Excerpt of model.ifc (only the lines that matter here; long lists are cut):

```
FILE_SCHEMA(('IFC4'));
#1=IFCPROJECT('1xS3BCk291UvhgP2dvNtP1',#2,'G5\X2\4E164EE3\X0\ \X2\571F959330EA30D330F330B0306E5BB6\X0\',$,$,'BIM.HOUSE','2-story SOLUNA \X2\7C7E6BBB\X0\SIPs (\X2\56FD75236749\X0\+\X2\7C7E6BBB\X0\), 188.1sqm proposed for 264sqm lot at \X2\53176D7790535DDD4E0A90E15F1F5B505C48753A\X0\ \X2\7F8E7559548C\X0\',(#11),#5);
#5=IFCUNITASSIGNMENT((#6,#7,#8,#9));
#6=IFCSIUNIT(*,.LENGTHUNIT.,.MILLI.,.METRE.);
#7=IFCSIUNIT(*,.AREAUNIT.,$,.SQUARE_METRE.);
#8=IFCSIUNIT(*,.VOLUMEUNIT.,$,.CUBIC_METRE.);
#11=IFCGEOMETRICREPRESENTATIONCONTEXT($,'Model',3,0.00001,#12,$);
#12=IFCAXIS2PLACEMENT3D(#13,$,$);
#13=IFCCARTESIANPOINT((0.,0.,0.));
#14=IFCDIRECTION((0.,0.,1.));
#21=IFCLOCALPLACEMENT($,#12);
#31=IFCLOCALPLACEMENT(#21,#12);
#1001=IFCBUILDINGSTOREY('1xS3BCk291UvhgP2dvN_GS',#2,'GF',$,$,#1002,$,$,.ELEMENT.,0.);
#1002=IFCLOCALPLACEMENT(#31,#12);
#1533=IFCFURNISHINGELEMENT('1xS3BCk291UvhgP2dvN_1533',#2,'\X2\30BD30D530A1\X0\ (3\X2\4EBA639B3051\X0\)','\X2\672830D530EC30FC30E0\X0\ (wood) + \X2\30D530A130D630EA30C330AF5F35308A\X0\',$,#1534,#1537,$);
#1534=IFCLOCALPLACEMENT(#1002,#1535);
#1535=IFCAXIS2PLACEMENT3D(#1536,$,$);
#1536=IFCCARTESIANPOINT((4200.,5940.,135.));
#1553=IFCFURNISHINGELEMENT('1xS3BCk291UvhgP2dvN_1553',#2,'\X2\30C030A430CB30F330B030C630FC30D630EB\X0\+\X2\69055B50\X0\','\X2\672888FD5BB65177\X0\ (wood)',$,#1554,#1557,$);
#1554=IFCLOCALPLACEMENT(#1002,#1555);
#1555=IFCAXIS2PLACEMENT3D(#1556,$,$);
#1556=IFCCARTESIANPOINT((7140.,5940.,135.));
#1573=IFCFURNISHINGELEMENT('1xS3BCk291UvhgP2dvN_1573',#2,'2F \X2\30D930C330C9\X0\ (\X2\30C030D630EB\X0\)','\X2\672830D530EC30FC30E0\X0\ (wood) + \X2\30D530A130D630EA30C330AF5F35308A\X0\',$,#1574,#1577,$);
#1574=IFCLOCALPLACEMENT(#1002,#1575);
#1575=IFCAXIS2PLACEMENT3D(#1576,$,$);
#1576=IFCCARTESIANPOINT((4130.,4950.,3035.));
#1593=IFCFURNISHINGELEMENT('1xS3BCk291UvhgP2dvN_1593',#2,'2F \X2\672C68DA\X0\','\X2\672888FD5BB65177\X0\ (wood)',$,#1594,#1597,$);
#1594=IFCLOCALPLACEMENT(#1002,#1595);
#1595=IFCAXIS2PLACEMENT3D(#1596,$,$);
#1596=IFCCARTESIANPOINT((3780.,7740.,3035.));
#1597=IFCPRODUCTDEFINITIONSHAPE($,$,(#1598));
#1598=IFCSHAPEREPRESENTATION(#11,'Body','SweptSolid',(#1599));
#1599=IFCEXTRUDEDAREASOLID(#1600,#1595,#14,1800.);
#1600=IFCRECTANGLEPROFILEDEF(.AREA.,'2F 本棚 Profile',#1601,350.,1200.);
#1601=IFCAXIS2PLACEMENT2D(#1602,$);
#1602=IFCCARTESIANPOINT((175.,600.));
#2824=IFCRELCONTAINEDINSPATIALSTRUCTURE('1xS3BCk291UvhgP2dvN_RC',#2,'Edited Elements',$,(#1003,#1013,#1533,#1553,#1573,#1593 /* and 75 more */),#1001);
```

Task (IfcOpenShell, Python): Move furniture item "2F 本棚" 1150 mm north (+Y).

```python
import ifcopenshell
import ifcopenshell.api.geometry
import ifcopenshell.util.placement

model = ifcopenshell.open("model.ifc")

item = model.by_guid("1xS3BCk291UvhgP2dvN_1593")
matrix = ifcopenshell.util.placement.get_local_placement(item.ObjectPlacement)
matrix[1, 3] += 1150.0
ifcopenshell.api.geometry.edit_object_placement(model, product=item, matrix=matrix, is_si=False)

print(ifcopenshell.util.placement.get_local_placement(item.ObjectPlacement).round(3) + 0.0)

model.write("model_edited.ifc")
```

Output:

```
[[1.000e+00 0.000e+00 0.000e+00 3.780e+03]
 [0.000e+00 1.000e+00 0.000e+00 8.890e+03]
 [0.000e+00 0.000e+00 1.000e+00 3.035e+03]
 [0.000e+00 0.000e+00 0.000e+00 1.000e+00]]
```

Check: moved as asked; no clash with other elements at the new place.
